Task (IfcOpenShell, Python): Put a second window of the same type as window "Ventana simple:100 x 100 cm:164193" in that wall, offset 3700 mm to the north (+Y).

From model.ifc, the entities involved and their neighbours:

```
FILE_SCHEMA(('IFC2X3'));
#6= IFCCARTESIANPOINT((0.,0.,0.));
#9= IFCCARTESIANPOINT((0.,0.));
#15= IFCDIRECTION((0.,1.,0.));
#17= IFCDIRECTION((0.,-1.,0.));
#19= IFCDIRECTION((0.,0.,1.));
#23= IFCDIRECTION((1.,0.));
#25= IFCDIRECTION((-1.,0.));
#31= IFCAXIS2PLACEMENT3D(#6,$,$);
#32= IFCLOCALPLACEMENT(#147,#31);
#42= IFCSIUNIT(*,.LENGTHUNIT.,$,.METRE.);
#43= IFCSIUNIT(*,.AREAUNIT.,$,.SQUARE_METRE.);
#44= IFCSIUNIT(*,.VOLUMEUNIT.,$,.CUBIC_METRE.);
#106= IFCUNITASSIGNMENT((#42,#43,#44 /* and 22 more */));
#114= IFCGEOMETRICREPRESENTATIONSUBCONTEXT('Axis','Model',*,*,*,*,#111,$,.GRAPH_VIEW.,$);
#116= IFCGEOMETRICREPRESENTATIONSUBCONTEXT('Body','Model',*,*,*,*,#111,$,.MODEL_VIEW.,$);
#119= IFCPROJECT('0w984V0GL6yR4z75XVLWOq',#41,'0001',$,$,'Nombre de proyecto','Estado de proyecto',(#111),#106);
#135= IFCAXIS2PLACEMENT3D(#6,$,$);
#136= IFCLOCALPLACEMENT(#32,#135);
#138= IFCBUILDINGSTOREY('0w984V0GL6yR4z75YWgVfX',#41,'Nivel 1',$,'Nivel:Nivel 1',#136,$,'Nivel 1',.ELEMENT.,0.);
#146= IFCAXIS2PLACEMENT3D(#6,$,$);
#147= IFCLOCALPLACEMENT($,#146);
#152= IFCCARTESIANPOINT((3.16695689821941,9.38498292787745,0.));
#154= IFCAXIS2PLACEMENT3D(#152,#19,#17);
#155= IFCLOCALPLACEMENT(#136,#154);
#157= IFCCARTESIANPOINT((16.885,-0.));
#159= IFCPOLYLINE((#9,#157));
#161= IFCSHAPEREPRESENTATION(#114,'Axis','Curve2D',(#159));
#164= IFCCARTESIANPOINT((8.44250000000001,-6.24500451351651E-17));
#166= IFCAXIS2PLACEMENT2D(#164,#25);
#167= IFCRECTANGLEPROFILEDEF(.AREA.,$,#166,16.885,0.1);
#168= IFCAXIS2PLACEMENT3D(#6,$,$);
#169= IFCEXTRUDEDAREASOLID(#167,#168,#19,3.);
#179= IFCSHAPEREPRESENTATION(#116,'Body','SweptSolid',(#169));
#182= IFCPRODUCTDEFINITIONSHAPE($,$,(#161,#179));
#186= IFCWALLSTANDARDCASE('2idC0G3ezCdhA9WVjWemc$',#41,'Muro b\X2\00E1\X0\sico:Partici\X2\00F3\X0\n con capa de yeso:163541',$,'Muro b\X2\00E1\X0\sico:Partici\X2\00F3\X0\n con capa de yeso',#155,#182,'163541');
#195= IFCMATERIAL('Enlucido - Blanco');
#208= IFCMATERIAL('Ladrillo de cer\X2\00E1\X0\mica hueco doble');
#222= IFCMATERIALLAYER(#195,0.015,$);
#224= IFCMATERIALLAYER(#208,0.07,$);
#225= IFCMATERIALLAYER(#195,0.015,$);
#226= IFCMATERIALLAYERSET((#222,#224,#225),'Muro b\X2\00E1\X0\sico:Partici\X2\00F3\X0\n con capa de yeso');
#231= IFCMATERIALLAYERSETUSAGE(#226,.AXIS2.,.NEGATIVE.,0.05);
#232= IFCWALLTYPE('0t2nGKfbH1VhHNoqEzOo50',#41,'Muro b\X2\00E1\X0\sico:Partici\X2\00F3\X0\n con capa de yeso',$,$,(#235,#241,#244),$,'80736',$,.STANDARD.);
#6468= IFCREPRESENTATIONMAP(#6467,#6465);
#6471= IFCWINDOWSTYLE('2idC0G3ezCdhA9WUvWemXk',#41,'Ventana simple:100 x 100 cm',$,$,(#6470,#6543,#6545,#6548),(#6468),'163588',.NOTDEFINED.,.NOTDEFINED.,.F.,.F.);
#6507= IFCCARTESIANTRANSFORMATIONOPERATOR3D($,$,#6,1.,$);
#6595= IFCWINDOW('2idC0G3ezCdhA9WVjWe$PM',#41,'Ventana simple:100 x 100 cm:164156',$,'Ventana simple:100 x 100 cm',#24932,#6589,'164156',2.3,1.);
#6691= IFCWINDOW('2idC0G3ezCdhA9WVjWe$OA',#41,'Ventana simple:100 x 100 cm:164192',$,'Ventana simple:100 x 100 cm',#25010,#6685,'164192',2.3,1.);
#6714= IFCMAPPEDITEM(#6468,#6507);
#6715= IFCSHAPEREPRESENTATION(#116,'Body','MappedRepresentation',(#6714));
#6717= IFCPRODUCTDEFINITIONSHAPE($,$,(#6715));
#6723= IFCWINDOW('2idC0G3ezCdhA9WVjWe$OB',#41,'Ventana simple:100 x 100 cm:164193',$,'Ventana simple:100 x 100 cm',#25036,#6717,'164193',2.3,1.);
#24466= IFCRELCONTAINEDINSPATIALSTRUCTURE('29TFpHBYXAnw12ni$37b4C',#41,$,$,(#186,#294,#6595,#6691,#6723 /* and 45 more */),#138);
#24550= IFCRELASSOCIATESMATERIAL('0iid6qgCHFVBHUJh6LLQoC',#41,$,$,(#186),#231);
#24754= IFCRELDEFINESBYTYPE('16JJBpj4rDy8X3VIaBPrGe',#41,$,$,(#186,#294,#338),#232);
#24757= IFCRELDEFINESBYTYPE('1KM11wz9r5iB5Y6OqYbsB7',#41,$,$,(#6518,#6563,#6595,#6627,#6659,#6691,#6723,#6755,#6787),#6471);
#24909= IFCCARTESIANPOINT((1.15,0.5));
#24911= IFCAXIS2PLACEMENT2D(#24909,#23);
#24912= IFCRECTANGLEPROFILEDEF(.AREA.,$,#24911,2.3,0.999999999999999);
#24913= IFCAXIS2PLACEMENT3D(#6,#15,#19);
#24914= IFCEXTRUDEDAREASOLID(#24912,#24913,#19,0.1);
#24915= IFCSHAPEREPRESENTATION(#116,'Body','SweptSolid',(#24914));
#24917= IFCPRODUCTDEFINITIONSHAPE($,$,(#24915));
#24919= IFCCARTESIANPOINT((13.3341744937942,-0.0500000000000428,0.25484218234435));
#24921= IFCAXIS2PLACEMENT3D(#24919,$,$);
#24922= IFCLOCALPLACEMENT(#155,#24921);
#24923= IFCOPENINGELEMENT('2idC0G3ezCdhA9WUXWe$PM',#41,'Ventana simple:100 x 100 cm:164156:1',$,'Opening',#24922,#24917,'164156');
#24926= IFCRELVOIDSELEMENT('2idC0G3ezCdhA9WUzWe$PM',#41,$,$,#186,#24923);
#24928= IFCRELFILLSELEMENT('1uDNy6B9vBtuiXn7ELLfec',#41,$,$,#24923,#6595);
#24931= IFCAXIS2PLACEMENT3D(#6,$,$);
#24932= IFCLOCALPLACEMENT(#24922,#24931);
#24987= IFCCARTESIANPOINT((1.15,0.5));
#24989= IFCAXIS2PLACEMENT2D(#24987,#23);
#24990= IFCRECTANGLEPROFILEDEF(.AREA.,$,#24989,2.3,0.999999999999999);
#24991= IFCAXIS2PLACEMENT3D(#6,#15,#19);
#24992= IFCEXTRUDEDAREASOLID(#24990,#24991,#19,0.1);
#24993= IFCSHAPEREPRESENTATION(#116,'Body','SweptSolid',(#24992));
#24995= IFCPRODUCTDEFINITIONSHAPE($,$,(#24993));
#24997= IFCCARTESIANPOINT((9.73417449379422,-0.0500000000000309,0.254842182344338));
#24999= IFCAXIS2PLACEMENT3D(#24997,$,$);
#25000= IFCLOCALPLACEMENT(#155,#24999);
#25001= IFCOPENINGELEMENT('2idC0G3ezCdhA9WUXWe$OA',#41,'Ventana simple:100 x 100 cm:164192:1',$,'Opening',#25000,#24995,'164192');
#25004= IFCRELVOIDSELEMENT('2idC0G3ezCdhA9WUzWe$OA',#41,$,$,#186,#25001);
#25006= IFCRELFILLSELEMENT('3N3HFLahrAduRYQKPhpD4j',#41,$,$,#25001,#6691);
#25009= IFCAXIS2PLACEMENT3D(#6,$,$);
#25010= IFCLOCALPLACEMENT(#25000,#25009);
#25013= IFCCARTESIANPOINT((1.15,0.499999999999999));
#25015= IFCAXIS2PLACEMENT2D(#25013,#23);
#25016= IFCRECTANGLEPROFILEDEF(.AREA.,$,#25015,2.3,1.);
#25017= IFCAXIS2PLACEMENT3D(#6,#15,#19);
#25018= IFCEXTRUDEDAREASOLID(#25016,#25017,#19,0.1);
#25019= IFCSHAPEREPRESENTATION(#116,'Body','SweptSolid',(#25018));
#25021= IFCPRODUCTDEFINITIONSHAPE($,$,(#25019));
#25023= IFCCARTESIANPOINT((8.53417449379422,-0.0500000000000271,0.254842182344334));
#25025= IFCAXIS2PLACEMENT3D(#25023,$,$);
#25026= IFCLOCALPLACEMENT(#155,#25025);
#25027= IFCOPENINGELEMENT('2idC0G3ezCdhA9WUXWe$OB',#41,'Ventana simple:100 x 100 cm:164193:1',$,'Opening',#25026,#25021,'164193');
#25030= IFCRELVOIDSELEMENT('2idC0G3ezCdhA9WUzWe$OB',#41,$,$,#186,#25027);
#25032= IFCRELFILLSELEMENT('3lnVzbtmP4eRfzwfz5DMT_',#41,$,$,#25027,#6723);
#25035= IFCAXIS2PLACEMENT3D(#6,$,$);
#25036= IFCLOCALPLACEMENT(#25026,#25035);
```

```python
import ifcopenshell
import ifcopenshell.api.feature
import ifcopenshell.api.geometry
import ifcopenshell.api.root
import ifcopenshell.geom
import ifcopenshell.util.element
import ifcopenshell.util.placement
import ifcopenshell.util.shape
import ifcopenshell.util.unit

model = ifcopenshell.open("model.ifc")
unit_scale = ifcopenshell.util.unit.calculate_unit_scale(model)
settings = ifcopenshell.geom.settings()


def volume(element):
    """Net volume in cubic metres, openings subtracted."""
    shape = ifcopenshell.geom.create_shape(settings, element)
    return ifcopenshell.util.shape.get_volume(shape.geometry)


def reuse_history(source, copy):
    """copy_class also copies each property set's owner history, people and application; keep the originals."""
    for rel in copy.IsDefinedBy:
        if rel.is_a("IfcRelDefinesByProperties") and (history := rel.RelatingPropertyDefinition.OwnerHistory):
            rel.RelatingPropertyDefinition.OwnerHistory = source.OwnerHistory
            ifcopenshell.util.element.remove_deep2(model, history)


window = model.by_guid("2idC0G3ezCdhA9WVjWe$OB")
opening = window.FillsVoids[0].RelatingOpeningElement
wall = opening.VoidsElements[0].RelatingBuildingElement
before = volume(wall)
shift = ifcopenshell.util.placement.get_local_placement(wall.ObjectPlacement)[:3, 0] * -3.7 / unit_scale

# copy_class copies the void relationship, type, container and properties, but no geometry.
new_opening = ifcopenshell.api.root.copy_class(model, product=opening)
new_opening.Representation = ifcopenshell.util.element.copy_deep(
    model, opening.Representation, exclude=["IfcGeometricRepresentationContext", "IfcRepresentationMap"]
)
new_opening.Name = "Ventana simple:100 x 100 cm"
new_opening.Tag = None
new_window = ifcopenshell.api.root.copy_class(model, product=window)
new_window.Representation = ifcopenshell.util.element.copy_deep(
    model, window.Representation, exclude=["IfcGeometricRepresentationContext", "IfcRepresentationMap"]
)
new_window.Name = "Ventana simple:100 x 100 cm"
new_window.Tag = None
reuse_history(window, new_window)
fills = ifcopenshell.api.feature.add_filling(model, opening=new_opening, element=new_window)
fills.OwnerHistory = new_window.OwnerHistory  # required in IFC2X3

for old, new in ((opening, new_opening), (window, new_window)):
    matrix = ifcopenshell.util.placement.get_local_placement(old.ObjectPlacement)
    matrix[:3, 3] += shift
    ifcopenshell.api.geometry.edit_object_placement(model, product=new, matrix=matrix, is_si=False)

after = volume(wall)

print(f"wall volume {before:.3f} -> {after:.3f} m3")

model.write("model_v2.ifc")
```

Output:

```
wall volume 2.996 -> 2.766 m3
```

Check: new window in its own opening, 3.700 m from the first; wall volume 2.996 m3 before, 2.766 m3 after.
